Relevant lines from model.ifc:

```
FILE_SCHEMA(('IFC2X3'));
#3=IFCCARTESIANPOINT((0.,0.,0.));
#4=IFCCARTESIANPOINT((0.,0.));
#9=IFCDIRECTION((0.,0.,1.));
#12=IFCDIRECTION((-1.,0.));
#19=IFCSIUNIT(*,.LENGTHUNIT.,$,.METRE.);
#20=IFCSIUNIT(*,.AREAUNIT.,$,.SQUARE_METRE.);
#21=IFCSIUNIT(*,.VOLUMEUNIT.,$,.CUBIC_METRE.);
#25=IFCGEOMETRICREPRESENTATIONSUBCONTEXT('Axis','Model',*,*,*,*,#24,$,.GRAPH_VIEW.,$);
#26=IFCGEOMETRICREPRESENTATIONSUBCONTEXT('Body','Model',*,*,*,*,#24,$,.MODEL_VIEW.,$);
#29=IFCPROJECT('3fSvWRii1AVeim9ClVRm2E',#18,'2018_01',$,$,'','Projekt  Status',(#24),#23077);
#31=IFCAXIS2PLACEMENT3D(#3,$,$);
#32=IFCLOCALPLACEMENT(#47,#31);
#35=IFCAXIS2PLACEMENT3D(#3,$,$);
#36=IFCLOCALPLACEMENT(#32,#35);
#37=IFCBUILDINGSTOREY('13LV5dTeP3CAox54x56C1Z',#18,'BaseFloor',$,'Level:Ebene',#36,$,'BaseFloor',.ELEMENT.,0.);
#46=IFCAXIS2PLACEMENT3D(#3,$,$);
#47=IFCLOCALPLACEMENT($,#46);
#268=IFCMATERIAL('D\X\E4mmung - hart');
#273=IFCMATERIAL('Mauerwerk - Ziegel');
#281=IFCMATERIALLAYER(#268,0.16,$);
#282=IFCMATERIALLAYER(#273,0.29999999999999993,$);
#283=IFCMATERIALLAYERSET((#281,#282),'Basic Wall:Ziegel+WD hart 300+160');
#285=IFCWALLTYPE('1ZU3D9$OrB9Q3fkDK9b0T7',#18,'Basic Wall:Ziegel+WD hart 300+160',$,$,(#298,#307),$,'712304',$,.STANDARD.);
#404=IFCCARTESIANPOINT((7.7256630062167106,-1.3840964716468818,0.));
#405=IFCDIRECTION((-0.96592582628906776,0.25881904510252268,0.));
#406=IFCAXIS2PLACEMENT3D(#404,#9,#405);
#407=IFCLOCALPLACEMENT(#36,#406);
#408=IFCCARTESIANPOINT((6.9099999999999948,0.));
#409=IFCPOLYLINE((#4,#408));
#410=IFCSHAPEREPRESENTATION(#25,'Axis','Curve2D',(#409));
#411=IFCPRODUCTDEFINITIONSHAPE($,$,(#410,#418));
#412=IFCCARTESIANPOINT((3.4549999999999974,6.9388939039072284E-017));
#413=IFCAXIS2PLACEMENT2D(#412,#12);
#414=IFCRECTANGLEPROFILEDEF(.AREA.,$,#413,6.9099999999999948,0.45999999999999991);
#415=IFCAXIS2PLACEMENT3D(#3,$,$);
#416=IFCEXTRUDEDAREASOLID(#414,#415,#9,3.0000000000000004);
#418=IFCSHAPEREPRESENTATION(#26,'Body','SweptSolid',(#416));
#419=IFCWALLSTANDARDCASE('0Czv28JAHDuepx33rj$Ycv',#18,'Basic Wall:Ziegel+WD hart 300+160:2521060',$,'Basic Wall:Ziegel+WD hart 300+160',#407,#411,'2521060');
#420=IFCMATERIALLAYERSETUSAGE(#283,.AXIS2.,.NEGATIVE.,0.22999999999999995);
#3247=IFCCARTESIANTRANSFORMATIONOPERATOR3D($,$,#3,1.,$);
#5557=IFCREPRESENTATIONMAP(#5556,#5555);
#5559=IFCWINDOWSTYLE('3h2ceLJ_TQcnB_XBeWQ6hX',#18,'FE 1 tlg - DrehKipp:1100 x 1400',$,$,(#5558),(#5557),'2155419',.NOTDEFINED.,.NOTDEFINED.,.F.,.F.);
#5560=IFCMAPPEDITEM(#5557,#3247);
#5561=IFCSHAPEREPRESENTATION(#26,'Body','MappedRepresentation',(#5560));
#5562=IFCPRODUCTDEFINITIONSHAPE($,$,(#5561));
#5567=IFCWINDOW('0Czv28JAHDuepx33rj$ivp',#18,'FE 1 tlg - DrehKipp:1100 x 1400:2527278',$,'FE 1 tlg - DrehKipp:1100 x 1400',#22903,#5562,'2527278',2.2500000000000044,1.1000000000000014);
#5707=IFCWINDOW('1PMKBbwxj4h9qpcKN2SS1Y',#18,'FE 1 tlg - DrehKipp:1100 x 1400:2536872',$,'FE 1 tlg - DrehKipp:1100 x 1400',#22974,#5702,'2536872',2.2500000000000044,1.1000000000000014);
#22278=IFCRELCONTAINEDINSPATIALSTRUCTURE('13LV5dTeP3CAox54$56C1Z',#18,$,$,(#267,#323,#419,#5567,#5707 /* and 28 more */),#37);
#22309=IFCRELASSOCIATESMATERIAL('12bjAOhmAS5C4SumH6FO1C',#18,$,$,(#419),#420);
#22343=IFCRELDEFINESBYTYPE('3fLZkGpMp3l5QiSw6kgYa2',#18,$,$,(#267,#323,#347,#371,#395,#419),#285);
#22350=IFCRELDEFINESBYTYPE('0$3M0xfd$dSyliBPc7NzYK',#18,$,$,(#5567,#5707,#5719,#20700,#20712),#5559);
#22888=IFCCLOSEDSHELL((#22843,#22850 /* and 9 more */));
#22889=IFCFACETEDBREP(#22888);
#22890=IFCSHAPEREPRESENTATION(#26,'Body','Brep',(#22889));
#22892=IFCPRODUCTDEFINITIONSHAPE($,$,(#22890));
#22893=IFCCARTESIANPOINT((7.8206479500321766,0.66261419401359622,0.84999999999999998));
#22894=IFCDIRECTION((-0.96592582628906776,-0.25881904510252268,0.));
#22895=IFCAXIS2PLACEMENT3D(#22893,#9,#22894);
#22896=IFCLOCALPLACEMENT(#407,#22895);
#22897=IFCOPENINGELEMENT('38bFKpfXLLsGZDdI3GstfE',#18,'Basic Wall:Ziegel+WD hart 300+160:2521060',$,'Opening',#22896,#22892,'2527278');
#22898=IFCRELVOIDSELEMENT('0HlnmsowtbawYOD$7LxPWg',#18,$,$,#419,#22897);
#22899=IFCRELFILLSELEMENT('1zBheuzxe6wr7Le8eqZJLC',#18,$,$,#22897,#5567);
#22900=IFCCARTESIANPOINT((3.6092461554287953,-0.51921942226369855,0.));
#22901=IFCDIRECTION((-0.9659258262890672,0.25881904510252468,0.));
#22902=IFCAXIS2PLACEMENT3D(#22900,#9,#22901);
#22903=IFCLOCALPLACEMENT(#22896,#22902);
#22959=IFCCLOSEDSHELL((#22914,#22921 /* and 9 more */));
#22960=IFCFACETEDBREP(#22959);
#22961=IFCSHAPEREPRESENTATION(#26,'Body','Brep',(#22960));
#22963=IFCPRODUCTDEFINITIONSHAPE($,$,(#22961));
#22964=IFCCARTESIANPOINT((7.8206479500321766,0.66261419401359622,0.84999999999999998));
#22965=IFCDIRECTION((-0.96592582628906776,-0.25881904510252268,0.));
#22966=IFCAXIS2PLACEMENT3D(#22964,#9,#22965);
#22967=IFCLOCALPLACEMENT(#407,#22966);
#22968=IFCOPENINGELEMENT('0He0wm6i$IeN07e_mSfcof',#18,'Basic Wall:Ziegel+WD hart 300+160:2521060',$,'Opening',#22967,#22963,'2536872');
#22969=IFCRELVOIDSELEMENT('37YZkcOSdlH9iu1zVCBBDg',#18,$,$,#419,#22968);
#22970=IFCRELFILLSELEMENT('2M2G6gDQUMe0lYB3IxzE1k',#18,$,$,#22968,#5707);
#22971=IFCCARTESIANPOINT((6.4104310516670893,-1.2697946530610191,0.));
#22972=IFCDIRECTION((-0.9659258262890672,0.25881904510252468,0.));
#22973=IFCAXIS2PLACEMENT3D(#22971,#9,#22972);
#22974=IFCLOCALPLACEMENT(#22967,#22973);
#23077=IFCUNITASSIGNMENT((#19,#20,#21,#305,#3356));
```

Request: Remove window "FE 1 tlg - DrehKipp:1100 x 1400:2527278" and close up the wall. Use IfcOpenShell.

```python
import ifcopenshell
import ifcopenshell.api.feature
import ifcopenshell.api.root
import ifcopenshell.geom
import ifcopenshell.util.shape

model = ifcopenshell.open("model.ifc")
settings = ifcopenshell.geom.settings()


def volume(element):
    """Net volume in cubic metres, openings subtracted."""
    shape = ifcopenshell.geom.create_shape(settings, element)
    return ifcopenshell.util.shape.get_volume(shape.geometry)


window = model.by_guid("0Czv28JAHDuepx33rj$ivp")
opening = window.FillsVoids[0].RelatingOpeningElement
wall = opening.VoidsElements[0].RelatingBuildingElement
before = volume(wall)

ifcopenshell.api.root.remove_product(model, product=window)
ifcopenshell.api.feature.remove_feature(model, feature=opening)

after = volume(wall)

print(f"wall volume {before:.3f} -> {after:.3f} m3")

model.write("model_rev.ifc")
```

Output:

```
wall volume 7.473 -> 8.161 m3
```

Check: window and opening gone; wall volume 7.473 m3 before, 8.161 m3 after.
